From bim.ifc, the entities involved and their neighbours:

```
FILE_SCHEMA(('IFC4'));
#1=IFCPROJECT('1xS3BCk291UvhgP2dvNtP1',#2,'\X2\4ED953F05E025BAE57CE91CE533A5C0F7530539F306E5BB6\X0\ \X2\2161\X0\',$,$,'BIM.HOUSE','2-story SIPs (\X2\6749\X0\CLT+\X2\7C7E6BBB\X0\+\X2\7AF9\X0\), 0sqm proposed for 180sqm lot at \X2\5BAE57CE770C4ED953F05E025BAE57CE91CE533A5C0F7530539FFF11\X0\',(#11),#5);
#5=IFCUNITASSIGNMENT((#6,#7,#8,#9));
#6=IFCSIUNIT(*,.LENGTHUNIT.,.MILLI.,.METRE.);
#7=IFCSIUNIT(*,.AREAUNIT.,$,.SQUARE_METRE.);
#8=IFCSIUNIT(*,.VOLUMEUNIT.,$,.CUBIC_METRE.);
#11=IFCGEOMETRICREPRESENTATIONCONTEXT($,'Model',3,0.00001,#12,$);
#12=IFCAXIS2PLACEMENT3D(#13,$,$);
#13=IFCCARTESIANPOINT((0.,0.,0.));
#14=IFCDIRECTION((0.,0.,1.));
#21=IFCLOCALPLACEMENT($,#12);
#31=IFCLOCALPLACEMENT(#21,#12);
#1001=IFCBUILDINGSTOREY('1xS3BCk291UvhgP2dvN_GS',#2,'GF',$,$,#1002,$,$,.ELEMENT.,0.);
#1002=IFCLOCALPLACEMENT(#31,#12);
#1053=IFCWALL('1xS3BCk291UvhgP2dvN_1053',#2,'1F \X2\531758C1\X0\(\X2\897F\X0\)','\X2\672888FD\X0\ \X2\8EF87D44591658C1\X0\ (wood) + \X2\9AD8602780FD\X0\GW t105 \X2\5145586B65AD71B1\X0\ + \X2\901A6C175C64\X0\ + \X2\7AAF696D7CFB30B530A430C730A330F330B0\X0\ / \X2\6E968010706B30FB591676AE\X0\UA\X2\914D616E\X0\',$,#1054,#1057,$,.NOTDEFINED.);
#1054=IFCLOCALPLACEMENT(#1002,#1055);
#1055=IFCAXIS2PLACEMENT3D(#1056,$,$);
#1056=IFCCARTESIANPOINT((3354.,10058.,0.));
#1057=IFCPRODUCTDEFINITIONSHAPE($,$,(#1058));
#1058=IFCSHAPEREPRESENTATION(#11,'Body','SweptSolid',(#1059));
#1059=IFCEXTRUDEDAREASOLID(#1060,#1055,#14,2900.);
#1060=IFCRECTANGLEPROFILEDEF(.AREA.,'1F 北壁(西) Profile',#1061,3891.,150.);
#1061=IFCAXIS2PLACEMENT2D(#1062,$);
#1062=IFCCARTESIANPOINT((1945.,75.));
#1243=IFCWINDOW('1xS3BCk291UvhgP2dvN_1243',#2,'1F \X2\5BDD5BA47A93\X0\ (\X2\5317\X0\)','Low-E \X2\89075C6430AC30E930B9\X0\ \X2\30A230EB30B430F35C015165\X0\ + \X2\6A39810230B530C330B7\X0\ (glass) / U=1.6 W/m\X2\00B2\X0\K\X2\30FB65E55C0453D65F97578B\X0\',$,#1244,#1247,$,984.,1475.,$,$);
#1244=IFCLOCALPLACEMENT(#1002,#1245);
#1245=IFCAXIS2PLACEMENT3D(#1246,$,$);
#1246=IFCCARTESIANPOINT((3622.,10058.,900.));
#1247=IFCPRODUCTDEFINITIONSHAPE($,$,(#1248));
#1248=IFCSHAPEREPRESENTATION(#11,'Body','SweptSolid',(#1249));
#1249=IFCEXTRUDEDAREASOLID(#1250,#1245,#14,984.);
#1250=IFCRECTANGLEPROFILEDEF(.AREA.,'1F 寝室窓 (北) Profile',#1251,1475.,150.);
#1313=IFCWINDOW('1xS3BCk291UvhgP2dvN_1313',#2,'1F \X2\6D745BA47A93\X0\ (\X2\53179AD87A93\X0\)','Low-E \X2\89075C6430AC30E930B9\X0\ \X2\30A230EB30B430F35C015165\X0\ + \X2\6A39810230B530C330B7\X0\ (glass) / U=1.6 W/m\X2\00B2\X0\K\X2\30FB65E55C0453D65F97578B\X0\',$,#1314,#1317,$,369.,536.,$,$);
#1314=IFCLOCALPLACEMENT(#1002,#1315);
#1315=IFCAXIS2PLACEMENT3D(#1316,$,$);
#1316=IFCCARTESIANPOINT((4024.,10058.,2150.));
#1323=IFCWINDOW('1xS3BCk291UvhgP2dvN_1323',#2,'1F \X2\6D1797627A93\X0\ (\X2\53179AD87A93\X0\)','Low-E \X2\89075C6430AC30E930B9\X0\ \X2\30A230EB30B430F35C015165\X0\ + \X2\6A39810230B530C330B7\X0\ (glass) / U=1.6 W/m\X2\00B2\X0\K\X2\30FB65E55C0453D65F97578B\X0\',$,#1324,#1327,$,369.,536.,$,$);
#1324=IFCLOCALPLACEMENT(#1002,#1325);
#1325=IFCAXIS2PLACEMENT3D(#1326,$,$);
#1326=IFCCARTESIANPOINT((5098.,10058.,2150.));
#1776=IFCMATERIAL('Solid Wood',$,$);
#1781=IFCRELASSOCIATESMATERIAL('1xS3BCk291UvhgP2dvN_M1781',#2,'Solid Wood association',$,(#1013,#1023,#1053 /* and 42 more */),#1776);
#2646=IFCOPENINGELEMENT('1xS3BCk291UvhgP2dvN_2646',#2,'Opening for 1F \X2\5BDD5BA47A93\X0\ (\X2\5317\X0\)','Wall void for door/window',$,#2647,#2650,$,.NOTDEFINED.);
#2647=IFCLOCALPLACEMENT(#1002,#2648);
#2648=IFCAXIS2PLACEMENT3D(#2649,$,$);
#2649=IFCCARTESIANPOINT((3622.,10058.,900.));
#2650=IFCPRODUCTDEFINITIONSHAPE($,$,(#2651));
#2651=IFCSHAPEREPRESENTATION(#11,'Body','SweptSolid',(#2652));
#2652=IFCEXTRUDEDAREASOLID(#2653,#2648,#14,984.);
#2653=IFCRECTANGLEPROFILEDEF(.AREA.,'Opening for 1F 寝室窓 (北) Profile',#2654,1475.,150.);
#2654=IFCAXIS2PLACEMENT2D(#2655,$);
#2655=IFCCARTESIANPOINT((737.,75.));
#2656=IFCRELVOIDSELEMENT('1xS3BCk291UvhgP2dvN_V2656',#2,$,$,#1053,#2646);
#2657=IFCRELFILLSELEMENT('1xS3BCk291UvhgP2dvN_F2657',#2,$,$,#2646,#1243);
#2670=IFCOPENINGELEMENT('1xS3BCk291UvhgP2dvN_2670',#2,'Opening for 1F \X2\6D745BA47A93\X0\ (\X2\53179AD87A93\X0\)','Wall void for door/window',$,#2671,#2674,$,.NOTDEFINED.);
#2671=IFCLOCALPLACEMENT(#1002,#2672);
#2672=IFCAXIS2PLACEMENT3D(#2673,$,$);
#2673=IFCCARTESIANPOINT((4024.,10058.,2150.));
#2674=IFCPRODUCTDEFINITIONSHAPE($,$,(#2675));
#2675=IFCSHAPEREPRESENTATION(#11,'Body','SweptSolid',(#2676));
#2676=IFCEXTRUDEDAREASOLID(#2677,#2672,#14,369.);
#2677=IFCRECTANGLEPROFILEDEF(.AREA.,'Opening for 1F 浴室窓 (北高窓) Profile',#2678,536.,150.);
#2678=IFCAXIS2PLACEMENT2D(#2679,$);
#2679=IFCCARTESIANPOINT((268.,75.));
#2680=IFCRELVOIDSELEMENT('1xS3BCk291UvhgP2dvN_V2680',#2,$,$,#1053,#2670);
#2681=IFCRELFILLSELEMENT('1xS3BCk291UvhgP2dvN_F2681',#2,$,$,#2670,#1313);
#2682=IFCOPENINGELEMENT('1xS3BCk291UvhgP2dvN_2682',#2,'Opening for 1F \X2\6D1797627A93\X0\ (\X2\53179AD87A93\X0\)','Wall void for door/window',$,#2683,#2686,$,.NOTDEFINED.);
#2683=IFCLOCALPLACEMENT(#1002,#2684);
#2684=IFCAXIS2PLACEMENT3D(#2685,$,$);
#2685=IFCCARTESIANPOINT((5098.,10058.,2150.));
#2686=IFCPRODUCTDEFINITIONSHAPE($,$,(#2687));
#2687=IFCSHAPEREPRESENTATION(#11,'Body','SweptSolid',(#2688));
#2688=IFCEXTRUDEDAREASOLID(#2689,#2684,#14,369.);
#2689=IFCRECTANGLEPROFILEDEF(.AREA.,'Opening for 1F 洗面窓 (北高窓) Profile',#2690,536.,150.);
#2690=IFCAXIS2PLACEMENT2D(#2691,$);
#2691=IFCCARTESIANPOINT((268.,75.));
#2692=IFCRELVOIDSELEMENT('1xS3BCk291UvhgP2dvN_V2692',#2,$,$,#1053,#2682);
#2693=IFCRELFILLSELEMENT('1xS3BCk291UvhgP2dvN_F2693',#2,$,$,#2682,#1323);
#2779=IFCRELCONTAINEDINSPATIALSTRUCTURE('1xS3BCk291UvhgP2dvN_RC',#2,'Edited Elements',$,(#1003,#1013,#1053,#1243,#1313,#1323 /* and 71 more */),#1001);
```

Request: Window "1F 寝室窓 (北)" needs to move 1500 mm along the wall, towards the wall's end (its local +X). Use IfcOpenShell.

```python
import ifcopenshell
import ifcopenshell.api.geometry
import ifcopenshell.util.placement

model = ifcopenshell.open("bim.ifc")

window = model.by_id(1243)
opening = window.FillsVoids[0].RelatingOpeningElement
wall = opening.VoidsElements[0].RelatingBuildingElement

wall_matrix = ifcopenshell.util.placement.get_local_placement(wall.ObjectPlacement)
shift = wall_matrix[:3, 0] * 1500.0
before = ifcopenshell.util.placement.get_local_placement(window.ObjectPlacement)[:3, 3].copy()

# The window is not placed relative to its opening, so move both.
for product in (opening, window):
    matrix = ifcopenshell.util.placement.get_local_placement(product.ObjectPlacement)
    matrix[:3, 3] += shift
    ifcopenshell.api.geometry.edit_object_placement(model, product=product, matrix=matrix, is_si=False)

after = ifcopenshell.util.placement.get_local_placement(window.ObjectPlacement)[:3, 3]
print("window moved by", (after - before).round(3) + 0.0)

model.write("bim_rev.ifc")
```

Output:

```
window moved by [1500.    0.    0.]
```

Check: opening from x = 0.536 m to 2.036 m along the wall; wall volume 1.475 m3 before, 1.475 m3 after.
